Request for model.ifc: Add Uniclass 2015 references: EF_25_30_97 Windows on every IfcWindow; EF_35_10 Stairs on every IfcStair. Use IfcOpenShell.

First a look at what the model holds.

```python
import ifcopenshell

model = ifcopenshell.open("model.ifc")
print(model.schema)
print("classifications:", [c.Name for c in model.by_type("IfcClassification")])
for ifc_class in ("IfcDoor", "IfcRoof", "IfcStair", "IfcWall", "IfcWindow"):
    print(ifc_class, len(model.by_type(ifc_class)))
```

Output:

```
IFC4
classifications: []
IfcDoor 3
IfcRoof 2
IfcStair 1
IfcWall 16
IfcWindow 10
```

```python
import ifcopenshell
import ifcopenshell.api.classification

model = ifcopenshell.open("model.ifc")

system = ifcopenshell.api.classification.add_classification(model, classification="Uniclass 2015")

codes = {
    "IfcWindow": ("EF_25_30_97", "Windows"),
    "IfcStair": ("EF_35_10", "Stairs"),
}
for ifc_class, (code, name) in codes.items():
    products = model.by_type(ifc_class)
    ifcopenshell.api.classification.add_reference(
        model, products=products, classification=system, identification=code, name=name
    )
    print(code, len(products))

model.write("model-out.ifc")
```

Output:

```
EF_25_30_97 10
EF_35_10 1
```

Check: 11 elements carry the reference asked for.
